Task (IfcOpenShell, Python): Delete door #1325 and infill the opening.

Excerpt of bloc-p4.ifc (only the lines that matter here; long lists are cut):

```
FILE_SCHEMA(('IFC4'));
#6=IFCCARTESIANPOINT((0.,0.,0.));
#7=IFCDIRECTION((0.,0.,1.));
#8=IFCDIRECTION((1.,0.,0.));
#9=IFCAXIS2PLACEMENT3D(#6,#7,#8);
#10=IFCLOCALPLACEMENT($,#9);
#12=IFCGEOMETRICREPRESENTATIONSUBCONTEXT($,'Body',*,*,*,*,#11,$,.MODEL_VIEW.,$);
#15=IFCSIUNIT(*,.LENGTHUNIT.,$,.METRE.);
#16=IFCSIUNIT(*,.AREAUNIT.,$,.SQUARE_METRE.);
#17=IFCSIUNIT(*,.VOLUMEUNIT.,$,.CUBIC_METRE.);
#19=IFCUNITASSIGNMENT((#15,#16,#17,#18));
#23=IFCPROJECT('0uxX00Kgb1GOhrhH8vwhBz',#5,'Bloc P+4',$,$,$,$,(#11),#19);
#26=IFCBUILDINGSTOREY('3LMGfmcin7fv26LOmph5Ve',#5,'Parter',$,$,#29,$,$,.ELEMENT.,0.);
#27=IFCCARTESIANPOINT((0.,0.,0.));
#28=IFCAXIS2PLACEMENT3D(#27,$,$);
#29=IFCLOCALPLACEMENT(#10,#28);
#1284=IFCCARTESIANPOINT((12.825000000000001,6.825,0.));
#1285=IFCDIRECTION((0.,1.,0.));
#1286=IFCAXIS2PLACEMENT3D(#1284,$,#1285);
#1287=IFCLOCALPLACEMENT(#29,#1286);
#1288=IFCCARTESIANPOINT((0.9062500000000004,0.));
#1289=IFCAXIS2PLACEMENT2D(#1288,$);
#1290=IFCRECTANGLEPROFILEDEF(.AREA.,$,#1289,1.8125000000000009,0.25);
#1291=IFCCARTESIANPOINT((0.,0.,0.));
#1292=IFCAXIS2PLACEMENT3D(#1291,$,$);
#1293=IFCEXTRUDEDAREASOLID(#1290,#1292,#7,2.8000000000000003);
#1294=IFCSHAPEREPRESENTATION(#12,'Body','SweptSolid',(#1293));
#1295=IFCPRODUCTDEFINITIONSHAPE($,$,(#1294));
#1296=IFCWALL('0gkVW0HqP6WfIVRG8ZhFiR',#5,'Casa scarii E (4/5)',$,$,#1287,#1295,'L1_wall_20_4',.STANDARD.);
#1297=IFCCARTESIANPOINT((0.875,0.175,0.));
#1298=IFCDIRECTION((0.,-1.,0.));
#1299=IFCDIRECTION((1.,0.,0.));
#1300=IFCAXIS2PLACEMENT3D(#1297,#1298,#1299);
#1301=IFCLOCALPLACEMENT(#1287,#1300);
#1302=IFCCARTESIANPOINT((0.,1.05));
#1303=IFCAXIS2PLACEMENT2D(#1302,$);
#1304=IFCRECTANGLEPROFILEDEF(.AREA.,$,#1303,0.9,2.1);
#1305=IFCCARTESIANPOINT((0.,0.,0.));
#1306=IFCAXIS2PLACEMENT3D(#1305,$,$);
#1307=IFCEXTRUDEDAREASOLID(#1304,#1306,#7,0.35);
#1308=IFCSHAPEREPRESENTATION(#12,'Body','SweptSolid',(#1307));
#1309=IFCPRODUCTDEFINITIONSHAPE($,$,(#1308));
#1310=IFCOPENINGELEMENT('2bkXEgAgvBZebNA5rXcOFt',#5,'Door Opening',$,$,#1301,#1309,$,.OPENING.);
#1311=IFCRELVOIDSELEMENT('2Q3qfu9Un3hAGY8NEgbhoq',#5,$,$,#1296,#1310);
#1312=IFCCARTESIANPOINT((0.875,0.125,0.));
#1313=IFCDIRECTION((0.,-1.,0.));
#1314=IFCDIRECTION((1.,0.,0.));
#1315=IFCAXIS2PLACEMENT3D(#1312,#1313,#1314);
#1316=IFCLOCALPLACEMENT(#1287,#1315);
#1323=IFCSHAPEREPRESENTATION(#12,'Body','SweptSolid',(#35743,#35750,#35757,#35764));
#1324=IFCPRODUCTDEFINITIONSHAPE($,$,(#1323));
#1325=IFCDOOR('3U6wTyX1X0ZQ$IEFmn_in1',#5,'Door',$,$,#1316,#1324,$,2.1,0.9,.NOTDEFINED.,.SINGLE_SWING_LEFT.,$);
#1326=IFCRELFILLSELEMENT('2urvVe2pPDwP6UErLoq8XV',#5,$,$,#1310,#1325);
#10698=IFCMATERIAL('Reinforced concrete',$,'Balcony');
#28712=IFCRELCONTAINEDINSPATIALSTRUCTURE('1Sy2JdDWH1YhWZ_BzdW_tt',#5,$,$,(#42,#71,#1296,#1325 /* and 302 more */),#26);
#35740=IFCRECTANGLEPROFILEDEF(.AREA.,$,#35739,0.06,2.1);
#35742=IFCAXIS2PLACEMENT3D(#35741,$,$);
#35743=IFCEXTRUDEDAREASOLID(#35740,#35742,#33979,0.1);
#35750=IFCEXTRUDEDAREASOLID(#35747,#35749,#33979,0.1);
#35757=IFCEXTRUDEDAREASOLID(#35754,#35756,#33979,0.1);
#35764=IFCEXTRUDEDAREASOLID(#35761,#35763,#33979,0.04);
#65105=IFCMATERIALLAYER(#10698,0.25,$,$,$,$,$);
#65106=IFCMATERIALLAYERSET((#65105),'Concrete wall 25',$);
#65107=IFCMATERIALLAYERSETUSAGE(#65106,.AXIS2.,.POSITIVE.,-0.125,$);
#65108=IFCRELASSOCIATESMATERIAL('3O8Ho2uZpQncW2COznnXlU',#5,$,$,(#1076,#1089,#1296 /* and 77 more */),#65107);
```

```python
import ifcopenshell
import ifcopenshell.api.feature
import ifcopenshell.api.root
import ifcopenshell.geom
import ifcopenshell.util.shape

model = ifcopenshell.open("bloc-p4.ifc")
settings = ifcopenshell.geom.settings()


def volume(element):
    """Net volume in cubic metres, openings subtracted."""
    shape = ifcopenshell.geom.create_shape(settings, element)
    return ifcopenshell.util.shape.get_volume(shape.geometry)


door = model.by_guid("3U6wTyX1X0ZQ$IEFmn_in1")
opening = door.FillsVoids[0].RelatingOpeningElement
wall = opening.VoidsElements[0].RelatingBuildingElement
before = volume(wall)

ifcopenshell.api.root.remove_product(model, product=door)
ifcopenshell.api.feature.remove_feature(model, feature=opening)

after = volume(wall)

print(f"wall volume {before:.3f} -> {after:.3f} m3")

model.write("bloc-p4-out.ifc")
```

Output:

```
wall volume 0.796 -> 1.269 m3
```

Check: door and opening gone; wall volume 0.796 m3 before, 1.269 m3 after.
